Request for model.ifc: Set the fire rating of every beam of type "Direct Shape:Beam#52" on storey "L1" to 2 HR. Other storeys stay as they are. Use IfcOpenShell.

First a look at what the model holds.

```python
import ifcopenshell
import ifcopenshell.util.element

model = ifcopenshell.open("model.ifc")
print(model.schema)
storey = next(s for s in model.by_type("IfcBuildingStorey") if s.Name == "L1")
beams = [e for e in ifcopenshell.util.element.get_decomposition(storey) if e.is_a("IfcBeam")]
seen = {}
for e in beams:
    element_type = ifcopenshell.util.element.get_type(e)
    key = (element_type.Name if element_type != e and element_type else None, ifcopenshell.util.element.get_pset(e, "Pset_BeamCommon", "FireRating"))
    seen[key] = seen.get(key, 0) + 1
for (name, value), count in sorted(seen.items(), key=str):
    print(count, "x", name, "|", value)
```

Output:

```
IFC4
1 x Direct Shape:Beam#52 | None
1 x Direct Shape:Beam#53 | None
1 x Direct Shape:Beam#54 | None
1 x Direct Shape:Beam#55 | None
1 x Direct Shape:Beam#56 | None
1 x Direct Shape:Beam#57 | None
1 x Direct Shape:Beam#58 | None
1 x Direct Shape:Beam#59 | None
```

```python
import ifcopenshell
import ifcopenshell.api.pset
import ifcopenshell.util.element

model = ifcopenshell.open("model.ifc")

storey = next(s for s in model.by_type("IfcBuildingStorey") if s.Name == "L1")
beams = [e for e in ifcopenshell.util.element.get_decomposition(storey) if e.is_a("IfcBeam")]

count = 0
for e in beams:
    element_type = ifcopenshell.util.element.get_type(e)
    if element_type in (None, e) or element_type.Name != "Direct Shape:Beam#52":
        continue
    # add_pset returns the element's existing set when there is one.
    pset = ifcopenshell.api.pset.add_pset(model, product=e, name="Pset_BeamCommon")
    ifcopenshell.api.pset.edit_pset(model, pset=pset, properties={"FireRating": "2 HR"})
    count += 1

print(count, "beams updated")

model.write("model-out.ifc")
```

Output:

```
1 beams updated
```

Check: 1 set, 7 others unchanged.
